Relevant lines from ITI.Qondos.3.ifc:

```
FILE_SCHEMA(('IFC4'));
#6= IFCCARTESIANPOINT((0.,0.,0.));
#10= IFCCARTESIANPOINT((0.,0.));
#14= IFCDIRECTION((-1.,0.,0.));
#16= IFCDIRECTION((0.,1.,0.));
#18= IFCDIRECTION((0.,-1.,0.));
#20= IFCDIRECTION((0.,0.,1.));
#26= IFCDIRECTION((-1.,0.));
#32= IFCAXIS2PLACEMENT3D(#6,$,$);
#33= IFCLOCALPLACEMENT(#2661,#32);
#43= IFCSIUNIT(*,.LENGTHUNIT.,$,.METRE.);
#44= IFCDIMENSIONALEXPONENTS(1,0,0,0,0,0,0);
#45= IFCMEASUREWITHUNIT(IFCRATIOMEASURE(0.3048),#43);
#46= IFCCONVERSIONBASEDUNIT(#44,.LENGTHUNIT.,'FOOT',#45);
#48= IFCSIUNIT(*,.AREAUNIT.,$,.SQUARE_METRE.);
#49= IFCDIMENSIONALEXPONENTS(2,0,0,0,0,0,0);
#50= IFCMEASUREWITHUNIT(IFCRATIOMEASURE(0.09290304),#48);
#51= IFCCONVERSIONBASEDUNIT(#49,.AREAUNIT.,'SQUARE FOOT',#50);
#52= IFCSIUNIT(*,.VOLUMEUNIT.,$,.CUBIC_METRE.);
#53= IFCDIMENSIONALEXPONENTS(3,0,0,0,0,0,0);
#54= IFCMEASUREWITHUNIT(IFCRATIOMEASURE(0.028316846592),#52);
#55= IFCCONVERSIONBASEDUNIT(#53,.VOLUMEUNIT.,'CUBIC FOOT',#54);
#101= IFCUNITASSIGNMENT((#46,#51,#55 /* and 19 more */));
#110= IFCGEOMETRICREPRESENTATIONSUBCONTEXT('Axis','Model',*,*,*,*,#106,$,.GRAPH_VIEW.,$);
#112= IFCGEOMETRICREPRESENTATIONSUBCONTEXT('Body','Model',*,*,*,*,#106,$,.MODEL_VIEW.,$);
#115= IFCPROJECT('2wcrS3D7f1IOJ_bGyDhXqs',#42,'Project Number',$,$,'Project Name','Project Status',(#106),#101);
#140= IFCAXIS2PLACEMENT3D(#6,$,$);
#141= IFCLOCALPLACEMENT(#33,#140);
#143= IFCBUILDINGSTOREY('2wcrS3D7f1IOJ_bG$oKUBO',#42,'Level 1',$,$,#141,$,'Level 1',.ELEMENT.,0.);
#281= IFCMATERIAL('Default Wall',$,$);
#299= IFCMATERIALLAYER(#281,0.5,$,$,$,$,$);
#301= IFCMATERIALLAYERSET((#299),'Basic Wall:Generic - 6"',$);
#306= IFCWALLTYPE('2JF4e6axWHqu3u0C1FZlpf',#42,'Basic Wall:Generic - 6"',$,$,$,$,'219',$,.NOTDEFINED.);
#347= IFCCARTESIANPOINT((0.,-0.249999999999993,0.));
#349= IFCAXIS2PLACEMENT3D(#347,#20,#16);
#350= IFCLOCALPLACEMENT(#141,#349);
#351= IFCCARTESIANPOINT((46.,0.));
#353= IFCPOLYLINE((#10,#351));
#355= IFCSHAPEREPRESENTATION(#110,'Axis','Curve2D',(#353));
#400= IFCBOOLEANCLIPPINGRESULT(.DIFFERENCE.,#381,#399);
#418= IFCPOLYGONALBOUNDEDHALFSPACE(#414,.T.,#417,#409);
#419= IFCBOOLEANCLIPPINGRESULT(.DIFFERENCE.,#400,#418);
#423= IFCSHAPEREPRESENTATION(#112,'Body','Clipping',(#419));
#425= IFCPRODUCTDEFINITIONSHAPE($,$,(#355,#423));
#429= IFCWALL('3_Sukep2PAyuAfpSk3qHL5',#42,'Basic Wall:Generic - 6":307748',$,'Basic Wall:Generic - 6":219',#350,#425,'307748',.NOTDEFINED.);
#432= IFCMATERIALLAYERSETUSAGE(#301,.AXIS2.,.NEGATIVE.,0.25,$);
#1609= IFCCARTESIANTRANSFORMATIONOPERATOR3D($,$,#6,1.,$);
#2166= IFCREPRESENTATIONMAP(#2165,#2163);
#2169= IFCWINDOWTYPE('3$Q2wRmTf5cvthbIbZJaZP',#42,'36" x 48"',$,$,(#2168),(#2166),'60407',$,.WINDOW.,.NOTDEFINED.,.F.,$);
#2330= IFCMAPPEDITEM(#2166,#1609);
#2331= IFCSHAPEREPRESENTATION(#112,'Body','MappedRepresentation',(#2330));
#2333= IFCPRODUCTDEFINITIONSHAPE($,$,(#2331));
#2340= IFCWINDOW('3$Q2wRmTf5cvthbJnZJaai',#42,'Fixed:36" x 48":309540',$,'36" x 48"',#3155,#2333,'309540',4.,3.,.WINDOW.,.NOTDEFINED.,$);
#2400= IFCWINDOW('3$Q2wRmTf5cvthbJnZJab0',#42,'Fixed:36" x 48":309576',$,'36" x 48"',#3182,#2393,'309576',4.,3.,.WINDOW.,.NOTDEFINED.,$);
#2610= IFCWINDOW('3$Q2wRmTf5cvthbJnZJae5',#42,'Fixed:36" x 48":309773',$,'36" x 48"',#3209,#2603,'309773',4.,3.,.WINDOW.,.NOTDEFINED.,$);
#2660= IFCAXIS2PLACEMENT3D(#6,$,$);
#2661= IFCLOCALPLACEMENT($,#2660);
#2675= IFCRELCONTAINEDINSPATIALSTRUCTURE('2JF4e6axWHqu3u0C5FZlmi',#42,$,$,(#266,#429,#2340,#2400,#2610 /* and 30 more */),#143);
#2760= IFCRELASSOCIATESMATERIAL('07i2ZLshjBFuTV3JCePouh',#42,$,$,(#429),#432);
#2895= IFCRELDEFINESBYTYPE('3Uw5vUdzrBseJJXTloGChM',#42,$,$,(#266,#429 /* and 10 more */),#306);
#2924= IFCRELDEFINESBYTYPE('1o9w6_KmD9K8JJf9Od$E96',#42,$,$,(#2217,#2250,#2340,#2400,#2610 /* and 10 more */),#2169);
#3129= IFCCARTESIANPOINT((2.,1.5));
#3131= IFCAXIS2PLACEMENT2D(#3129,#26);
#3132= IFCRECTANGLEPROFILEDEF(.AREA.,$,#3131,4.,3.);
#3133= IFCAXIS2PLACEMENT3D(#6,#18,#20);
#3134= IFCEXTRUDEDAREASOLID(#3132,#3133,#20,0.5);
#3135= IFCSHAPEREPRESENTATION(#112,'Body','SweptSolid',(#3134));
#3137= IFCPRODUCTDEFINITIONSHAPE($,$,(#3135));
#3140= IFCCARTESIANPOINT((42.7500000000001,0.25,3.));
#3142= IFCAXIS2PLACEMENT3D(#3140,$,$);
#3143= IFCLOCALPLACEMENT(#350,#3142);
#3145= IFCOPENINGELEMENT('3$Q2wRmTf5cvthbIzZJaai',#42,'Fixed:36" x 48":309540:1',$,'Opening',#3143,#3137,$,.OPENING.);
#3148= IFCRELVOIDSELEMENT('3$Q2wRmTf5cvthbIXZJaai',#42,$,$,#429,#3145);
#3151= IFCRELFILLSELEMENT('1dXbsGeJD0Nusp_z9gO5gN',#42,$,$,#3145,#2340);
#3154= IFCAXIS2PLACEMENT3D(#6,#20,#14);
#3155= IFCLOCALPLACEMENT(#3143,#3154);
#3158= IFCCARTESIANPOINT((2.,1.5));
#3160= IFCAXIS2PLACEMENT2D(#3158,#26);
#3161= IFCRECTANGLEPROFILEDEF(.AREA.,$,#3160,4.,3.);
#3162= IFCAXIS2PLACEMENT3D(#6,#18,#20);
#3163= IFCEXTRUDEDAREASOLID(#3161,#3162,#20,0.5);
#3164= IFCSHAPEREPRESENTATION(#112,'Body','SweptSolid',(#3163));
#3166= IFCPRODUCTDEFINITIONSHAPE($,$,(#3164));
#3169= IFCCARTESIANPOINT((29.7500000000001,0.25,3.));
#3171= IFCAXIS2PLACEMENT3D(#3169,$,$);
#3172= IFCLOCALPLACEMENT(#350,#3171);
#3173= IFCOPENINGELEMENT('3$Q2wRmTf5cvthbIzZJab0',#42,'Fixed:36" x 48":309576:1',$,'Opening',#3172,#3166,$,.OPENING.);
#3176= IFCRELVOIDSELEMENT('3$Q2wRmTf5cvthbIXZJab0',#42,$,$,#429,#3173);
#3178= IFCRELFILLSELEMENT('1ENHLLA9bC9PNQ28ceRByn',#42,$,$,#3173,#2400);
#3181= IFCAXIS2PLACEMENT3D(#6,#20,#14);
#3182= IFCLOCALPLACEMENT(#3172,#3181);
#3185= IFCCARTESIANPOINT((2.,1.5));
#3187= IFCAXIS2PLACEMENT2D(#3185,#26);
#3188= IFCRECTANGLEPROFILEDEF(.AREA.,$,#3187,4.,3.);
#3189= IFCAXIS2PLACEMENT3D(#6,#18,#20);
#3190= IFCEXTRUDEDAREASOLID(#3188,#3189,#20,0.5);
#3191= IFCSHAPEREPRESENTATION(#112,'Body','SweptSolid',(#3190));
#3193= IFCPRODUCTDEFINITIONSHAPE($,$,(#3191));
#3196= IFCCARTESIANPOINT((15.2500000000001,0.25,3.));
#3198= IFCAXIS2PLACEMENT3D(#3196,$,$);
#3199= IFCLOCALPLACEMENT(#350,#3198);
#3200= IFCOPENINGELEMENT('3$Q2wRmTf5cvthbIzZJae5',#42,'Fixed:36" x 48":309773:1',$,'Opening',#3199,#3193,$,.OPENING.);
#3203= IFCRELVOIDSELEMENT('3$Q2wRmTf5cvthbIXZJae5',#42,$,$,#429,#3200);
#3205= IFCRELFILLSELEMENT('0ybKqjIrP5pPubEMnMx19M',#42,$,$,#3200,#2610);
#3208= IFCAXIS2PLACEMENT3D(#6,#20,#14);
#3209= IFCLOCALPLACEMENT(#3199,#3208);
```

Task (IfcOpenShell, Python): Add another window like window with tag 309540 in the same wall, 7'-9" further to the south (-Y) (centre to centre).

```python
import ifcopenshell
import ifcopenshell.api.feature
import ifcopenshell.api.geometry
import ifcopenshell.api.root
import ifcopenshell.geom
import ifcopenshell.util.element
import ifcopenshell.util.placement
import ifcopenshell.util.shape
import ifcopenshell.util.unit

model = ifcopenshell.open("ITI.Qondos.3.ifc")
unit_scale = ifcopenshell.util.unit.calculate_unit_scale(model)
settings = ifcopenshell.geom.settings()


def volume(element):
    """Net volume in cubic metres, openings subtracted."""
    shape = ifcopenshell.geom.create_shape(settings, element)
    return ifcopenshell.util.shape.get_volume(shape.geometry)


def reuse_history(source, copy):
    """copy_class also copies each property set's owner history, people and application; keep the originals."""
    for rel in copy.IsDefinedBy:
        if rel.is_a("IfcRelDefinesByProperties") and (history := rel.RelatingPropertyDefinition.OwnerHistory):
            rel.RelatingPropertyDefinition.OwnerHistory = source.OwnerHistory
            ifcopenshell.util.element.remove_deep2(model, history)


window = model.by_guid("3$Q2wRmTf5cvthbJnZJaai")
opening = window.FillsVoids[0].RelatingOpeningElement
wall = opening.VoidsElements[0].RelatingBuildingElement
before = volume(wall)
shift = ifcopenshell.util.placement.get_local_placement(wall.ObjectPlacement)[:3, 0] * -93 * 0.0254 / unit_scale

# copy_class copies the void relationship, type, container and properties, but no geometry.
new_opening = ifcopenshell.api.root.copy_class(model, product=opening)
new_opening.Representation = ifcopenshell.util.element.copy_deep(
    model, opening.Representation, exclude=["IfcGeometricRepresentationContext", "IfcRepresentationMap"]
)
new_opening.Name = 'Fixed:36" x 48"'
new_window = ifcopenshell.api.root.copy_class(model, product=window)
new_window.Representation = ifcopenshell.util.element.copy_deep(
    model, window.Representation, exclude=["IfcGeometricRepresentationContext", "IfcRepresentationMap"]
)
new_window.Name = 'Fixed:36" x 48"'
new_window.Tag = None
reuse_history(window, new_window)
ifcopenshell.api.feature.add_filling(model, opening=new_opening, element=new_window)

for old, new in ((opening, new_opening), (window, new_window)):
    matrix = ifcopenshell.util.placement.get_local_placement(old.ObjectPlacement)
    matrix[:3, 3] += shift
    ifcopenshell.api.geometry.edit_object_placement(model, product=new, matrix=matrix, is_si=False)

after = volume(wall)

print(f"wall volume {before:.3f} -> {after:.3f} m3")

model.write("ITI.Qondos.3_updated.ifc")
```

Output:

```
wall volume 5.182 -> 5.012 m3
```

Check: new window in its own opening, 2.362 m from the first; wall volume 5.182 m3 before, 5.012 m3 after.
